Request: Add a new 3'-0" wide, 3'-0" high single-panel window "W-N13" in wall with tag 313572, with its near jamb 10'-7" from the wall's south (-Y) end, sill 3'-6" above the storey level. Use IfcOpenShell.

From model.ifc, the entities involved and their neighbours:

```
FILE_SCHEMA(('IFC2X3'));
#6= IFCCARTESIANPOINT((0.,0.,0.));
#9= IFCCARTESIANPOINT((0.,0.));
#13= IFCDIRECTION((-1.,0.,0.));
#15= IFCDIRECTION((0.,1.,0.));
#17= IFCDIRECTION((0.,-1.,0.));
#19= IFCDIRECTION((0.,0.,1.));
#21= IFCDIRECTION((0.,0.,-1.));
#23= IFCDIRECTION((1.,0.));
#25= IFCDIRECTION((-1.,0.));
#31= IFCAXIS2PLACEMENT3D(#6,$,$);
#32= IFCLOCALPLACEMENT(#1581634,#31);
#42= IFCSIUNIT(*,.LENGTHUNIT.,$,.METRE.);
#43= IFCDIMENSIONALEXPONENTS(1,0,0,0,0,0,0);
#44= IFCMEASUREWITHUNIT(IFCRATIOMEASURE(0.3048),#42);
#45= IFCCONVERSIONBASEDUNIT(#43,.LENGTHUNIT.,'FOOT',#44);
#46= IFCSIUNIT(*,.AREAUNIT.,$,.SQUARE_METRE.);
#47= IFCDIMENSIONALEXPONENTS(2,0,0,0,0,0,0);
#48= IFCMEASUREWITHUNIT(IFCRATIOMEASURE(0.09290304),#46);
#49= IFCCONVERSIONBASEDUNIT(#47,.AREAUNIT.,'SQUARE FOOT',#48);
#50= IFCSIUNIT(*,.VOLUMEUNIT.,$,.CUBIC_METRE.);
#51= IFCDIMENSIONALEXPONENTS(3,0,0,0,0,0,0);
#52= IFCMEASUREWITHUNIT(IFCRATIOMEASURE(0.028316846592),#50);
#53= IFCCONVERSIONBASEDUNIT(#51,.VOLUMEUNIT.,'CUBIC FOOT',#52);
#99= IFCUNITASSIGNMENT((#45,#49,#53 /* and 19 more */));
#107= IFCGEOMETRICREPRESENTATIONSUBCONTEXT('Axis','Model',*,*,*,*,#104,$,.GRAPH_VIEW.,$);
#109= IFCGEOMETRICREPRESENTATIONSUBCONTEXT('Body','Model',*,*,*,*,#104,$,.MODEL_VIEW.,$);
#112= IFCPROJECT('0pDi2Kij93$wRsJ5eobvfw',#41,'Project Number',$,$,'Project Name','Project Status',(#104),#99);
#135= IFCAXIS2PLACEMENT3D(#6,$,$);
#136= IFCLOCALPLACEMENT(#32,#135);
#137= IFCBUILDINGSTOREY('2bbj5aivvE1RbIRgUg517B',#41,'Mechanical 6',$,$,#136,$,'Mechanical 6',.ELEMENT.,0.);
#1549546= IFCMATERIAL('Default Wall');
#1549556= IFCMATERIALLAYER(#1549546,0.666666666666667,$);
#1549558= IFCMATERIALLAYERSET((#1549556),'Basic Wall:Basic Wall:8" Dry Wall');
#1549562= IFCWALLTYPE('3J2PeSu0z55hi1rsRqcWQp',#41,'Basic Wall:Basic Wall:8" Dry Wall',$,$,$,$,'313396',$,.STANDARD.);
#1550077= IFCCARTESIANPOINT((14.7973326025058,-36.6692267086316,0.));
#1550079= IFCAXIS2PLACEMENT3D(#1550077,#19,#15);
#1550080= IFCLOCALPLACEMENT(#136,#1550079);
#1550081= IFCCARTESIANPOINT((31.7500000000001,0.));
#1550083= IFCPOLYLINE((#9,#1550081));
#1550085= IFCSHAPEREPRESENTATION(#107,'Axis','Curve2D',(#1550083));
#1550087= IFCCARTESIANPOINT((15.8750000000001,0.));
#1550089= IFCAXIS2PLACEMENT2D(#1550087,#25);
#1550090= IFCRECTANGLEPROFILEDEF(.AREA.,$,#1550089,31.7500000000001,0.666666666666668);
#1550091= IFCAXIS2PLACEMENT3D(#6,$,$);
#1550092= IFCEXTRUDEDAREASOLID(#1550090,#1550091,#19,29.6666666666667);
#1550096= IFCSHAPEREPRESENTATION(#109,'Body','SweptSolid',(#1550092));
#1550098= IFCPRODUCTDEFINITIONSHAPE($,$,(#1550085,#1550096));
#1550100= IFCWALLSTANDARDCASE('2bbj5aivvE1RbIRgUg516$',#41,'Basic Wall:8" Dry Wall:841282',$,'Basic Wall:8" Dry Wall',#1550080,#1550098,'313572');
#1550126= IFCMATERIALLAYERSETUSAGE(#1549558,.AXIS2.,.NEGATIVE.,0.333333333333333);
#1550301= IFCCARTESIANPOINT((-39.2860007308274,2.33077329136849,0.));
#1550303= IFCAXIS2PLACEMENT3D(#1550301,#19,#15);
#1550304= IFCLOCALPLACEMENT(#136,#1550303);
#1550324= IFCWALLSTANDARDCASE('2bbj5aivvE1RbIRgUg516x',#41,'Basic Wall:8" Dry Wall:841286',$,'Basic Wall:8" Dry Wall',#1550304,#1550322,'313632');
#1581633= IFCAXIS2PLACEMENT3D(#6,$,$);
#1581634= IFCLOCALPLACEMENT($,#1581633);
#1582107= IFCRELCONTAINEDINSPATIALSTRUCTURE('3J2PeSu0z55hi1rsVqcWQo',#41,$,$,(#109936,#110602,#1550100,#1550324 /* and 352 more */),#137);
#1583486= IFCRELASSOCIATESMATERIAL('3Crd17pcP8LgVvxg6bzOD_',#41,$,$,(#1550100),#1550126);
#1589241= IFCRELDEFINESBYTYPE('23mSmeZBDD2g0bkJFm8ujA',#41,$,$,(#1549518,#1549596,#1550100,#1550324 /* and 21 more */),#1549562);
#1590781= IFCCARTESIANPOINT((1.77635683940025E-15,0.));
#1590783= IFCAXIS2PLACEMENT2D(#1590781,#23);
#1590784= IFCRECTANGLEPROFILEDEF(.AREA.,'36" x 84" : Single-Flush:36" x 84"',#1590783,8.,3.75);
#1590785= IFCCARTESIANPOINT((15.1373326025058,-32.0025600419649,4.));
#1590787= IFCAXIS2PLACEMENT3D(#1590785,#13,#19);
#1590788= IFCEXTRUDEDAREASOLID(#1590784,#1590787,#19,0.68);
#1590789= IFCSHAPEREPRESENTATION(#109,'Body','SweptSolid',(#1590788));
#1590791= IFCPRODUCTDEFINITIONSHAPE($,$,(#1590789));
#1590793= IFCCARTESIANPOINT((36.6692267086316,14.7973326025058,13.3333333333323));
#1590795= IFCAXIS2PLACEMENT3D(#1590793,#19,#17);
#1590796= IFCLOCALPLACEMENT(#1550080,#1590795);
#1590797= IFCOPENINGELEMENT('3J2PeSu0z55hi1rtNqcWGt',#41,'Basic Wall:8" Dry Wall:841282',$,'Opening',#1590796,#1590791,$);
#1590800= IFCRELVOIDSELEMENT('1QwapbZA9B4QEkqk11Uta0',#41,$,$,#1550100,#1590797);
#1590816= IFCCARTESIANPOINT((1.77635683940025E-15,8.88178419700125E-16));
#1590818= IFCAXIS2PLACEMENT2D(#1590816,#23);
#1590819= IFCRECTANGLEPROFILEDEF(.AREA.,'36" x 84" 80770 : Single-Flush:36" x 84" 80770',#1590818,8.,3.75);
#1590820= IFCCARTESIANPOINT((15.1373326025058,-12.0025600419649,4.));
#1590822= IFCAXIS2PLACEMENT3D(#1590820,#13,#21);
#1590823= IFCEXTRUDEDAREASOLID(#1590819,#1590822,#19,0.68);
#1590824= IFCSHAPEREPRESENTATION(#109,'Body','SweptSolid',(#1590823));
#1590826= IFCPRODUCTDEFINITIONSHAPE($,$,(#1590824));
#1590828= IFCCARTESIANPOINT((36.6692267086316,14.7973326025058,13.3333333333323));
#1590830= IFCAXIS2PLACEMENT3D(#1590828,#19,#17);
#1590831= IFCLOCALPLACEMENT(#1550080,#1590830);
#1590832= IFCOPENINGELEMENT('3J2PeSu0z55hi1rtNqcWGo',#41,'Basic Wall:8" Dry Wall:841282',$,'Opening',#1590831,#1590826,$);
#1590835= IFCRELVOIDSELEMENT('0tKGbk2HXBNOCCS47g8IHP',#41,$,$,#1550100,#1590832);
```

```python
import numpy as np
import ifcopenshell
import ifcopenshell.api.feature
import ifcopenshell.api.geometry
import ifcopenshell.api.root
import ifcopenshell.api.spatial
import ifcopenshell.api.type
import ifcopenshell.geom
import ifcopenshell.util.element
import ifcopenshell.util.placement
import ifcopenshell.util.representation
import ifcopenshell.util.shape
import ifcopenshell.util.unit

model = ifcopenshell.open("model.ifc")
unit_scale = ifcopenshell.util.unit.calculate_unit_scale(model)
settings = ifcopenshell.geom.settings()


def volume(element):
    """Net volume in cubic metres, openings subtracted."""
    shape = ifcopenshell.geom.create_shape(settings, element)
    return ifcopenshell.util.shape.get_volume(shape.geometry)


wall = model.by_guid("2bbj5aivvE1RbIRgUg516$")
storey = ifcopenshell.util.element.get_container(wall, ifc_class="IfcBuildingStorey")
context = ifcopenshell.util.representation.get_context(model, "Model", "Body", "MODEL_VIEW")
before = volume(wall)

width, height, from_end, sill = 0.9144, 0.9144, 3.2258, 1.0668  # metres

# The wall runs along its own X axis, and the end named is its -X end.
wall_shape = ifcopenshell.geom.create_shape(settings, wall)
x, y, z = ifcopenshell.util.shape.get_vertices(wall_shape.geometry).T
start = x.min() + from_end
face, thickness = float(y.min()), float(y.max() - y.min())
wall_matrix = ifcopenshell.util.placement.get_local_placement(wall.ObjectPlacement)
level = ifcopenshell.util.placement.get_local_placement(storey.ObjectPlacement)[2, 3]


def in_wall(x, y):
    """Placement at x, y metres in the wall's axes, at sill height."""
    matrix = wall_matrix.copy()
    matrix[:, 3] = wall_matrix @ np.array([x / unit_scale, y / unit_scale, 0.0, 1.0])
    matrix[2, 3] = level + sill / unit_scale
    return matrix


# Opening: a box that overshoots both wall faces by 50 mm.
opening = ifcopenshell.api.root.create_entity(model, ifc_class="IfcOpeningElement")
box = ifcopenshell.api.geometry.add_wall_representation(
    model, context=context, length=width, height=height, thickness=thickness + 0.1
)
ifcopenshell.api.geometry.assign_representation(model, product=opening, representation=box)
ifcopenshell.api.geometry.edit_object_placement(model, product=opening, matrix=in_wall(start, face - 0.05), is_si=False)
ifcopenshell.api.feature.add_feature(model, feature=opening, element=wall)

window = ifcopenshell.api.root.create_entity(model, ifc_class="IfcWindow", name="W-N13")
window.OverallWidth, window.OverallHeight = width / unit_scale, height / unit_scale
body = ifcopenshell.api.geometry.add_window_representation(
    model,
    context=context,
    overall_width=window.OverallWidth,
    overall_height=window.OverallHeight,
    partition_type="SINGLE_PANEL",
)
ifcopenshell.api.geometry.assign_representation(model, product=window, representation=body)
ifcopenshell.api.spatial.assign_container(model, products=[window], relating_structure=storey)
fills = ifcopenshell.api.feature.add_filling(model, opening=opening, element=window)
fills.OwnerHistory = window.OwnerHistory  # required in IFC2X3

# IFC2X3 keeps the operation on the window style.
style = ifcopenshell.api.root.create_entity(model, ifc_class="IfcWindowStyle", name="W-N13")
style.OperationType, style.ConstructionType = "SINGLE_PANEL", "NOTDEFINED"
style.ParameterTakesPrecedence = style.Sizeable = False
ifcopenshell.api.type.assign_type(model, related_objects=[window], relating_type=style)

# Centre the window in the wall's thickness.
ifcopenshell.api.geometry.edit_object_placement(model, product=window, matrix=in_wall(start, face), is_si=False)
window_shape = ifcopenshell.geom.create_shape(settings, window)
depth = ifcopenshell.util.shape.get_vertices(window_shape.geometry)[:, 1]
offset = face + thickness / 2 - (depth.min() + depth.max()) / 2
ifcopenshell.api.geometry.edit_object_placement(model, product=window, matrix=in_wall(start, offset), is_si=False)

after = volume(wall)

print(f"wall volume {before:.3f} -> {after:.3f} m3")

model.write("model_rev.ifc")
```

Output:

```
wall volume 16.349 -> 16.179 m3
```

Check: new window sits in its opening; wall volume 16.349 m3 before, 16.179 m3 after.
